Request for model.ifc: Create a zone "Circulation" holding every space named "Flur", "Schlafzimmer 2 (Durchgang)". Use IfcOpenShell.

First a look at what the model holds.

```python
import ifcopenshell

model = ifcopenshell.open("model.ifc")
print(model.schema)
seen = {}
for space in model.by_type("IfcSpace"):
    seen[space.LongName] = seen.get(space.LongName, 0) + 1
for name, count in sorted(seen.items(), key=str):
    print(count, "x", name)
print("zones:", [z.Name for z in model.by_type("IfcZone")][:20])
```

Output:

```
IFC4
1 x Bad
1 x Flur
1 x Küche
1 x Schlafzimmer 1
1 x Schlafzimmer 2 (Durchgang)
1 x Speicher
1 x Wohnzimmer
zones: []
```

```python
import ifcopenshell
import ifcopenshell.api.group
import ifcopenshell.api.root

model = ifcopenshell.open("model.ifc")

names = {"Flur", "Schlafzimmer 2 (Durchgang)"}
spaces = [s for s in model.by_type("IfcSpace") if s.LongName in names]

zone = ifcopenshell.api.root.create_entity(model, ifc_class="IfcZone", name="Circulation")
ifcopenshell.api.group.assign_group(model, products=spaces, group=zone)
print(len(spaces), "spaces in", zone.Name)

model.write("model_v2.ifc")
```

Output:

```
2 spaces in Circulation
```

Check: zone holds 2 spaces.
